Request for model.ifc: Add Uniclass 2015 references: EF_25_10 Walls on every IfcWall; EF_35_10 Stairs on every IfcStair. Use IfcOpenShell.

First a look at what the model holds.

```python
import ifcopenshell

model = ifcopenshell.open("model.ifc")
print(model.schema)
print("classifications:", [c.Name for c in model.by_type("IfcClassification")])
for ifc_class in ("IfcDoor", "IfcRoof", "IfcStair", "IfcWall", "IfcWindow"):
    print(ifc_class, len(model.by_type(ifc_class)))
```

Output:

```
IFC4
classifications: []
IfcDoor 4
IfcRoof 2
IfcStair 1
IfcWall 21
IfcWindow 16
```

```python
import ifcopenshell
import ifcopenshell.api.classification

model = ifcopenshell.open("model.ifc")

system = ifcopenshell.api.classification.add_classification(model, classification="Uniclass 2015")

codes = {
    "IfcWall": ("EF_25_10", "Walls"),
    "IfcStair": ("EF_35_10", "Stairs"),
}
for ifc_class, (code, name) in codes.items():
    products = model.by_type(ifc_class)
    ifcopenshell.api.classification.add_reference(
        model, products=products, classification=system, identification=code, name=name
    )
    print(code, len(products))

model.write("model_edited.ifc")
```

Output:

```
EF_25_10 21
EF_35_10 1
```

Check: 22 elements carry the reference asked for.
